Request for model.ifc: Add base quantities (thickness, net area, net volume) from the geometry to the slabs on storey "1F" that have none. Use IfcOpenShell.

First a look at what the model holds.

```python
import ifcopenshell
import ifcopenshell.util.element
import ifcopenshell.util.unit

model = ifcopenshell.open("model.ifc")
print(model.schema)
for unit_type in ("LENGTHUNIT", "AREAUNIT", "VOLUMEUNIT"):
    print(unit_type, ifcopenshell.util.unit.calculate_unit_scale(model, unit_type))
storey = next(s for s in model.by_type("IfcBuildingStorey") if s.Name == "1F")
slabs = [e for e in ifcopenshell.util.element.get_decomposition(storey) if e.is_a("IfcSlab")]
for e in sorted(slabs, key=lambda e: e.id()):
    print(e.id(), e.is_a(), e.Name, list(ifcopenshell.util.element.get_psets(e, qtos_only=True)), sep=" | ")
```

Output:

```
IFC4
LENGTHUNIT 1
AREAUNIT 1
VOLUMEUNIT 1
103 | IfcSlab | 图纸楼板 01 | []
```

```python
import ifcopenshell
import ifcopenshell.api.pset
import ifcopenshell.geom
import ifcopenshell.util.element
import ifcopenshell.util.shape
import ifcopenshell.util.unit

model = ifcopenshell.open("model.ifc")
unit_scale = ifcopenshell.util.unit.calculate_unit_scale(model)
area_scale = ifcopenshell.util.unit.calculate_unit_scale(model, "AREAUNIT")
volume_scale = ifcopenshell.util.unit.calculate_unit_scale(model, "VOLUMEUNIT")
settings = ifcopenshell.geom.settings()

storey = next(s for s in model.by_type("IfcBuildingStorey") if s.Name == "1F")
slabs = [e for e in ifcopenshell.util.element.get_decomposition(storey) if e.is_a("IfcSlab")]

for e in sorted(slabs, key=lambda e: e.id()):
    if ifcopenshell.util.element.get_psets(e, qtos_only=True, should_inherit=False):
        continue
    # Geometry comes back in metres, in the element's own axes.
    shape = ifcopenshell.geom.create_shape(settings, e)
    values = {
        "Width": ifcopenshell.util.shape.get_z(shape.geometry) / unit_scale,
        "NetArea": ifcopenshell.util.shape.get_footprint_area(shape.geometry) / area_scale,
        "NetVolume": ifcopenshell.util.shape.get_volume(shape.geometry) / volume_scale,
    }
    qto = ifcopenshell.api.pset.add_qto(model, product=e, name="Qto_SlabBaseQuantities")
    ifcopenshell.api.pset.edit_qto(model, qto=qto, properties=values)
    print(e.id(), {k: round(v, 3) for k, v in values.items()})

model.write("model-out.ifc")
```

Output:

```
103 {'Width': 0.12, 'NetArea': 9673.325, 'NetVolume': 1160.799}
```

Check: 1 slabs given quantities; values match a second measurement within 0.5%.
